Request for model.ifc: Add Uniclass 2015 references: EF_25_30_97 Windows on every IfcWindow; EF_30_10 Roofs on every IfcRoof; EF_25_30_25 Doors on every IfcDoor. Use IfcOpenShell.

First a look at what the model holds.

```python
import ifcopenshell

model = ifcopenshell.open("model.ifc")
print(model.schema)
print("classifications:", [c.Name for c in model.by_type("IfcClassification")])
for ifc_class in ("IfcDoor", "IfcRoof", "IfcStair", "IfcWall", "IfcWindow"):
    print(ifc_class, len(model.by_type(ifc_class)))
```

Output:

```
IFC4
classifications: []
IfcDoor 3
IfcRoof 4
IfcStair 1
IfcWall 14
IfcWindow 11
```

```python
import ifcopenshell
import ifcopenshell.api.classification

model = ifcopenshell.open("model.ifc")

system = ifcopenshell.api.classification.add_classification(model, classification="Uniclass 2015")

codes = {
    "IfcWindow": ("EF_25_30_97", "Windows"),
    "IfcRoof": ("EF_30_10", "Roofs"),
    "IfcDoor": ("EF_25_30_25", "Doors"),
}
for ifc_class, (code, name) in codes.items():
    products = model.by_type(ifc_class)
    ifcopenshell.api.classification.add_reference(
        model, products=products, classification=system, identification=code, name=name
    )
    print(code, len(products))

model.write("model_edited.ifc")
```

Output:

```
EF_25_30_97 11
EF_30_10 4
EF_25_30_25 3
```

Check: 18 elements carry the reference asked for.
